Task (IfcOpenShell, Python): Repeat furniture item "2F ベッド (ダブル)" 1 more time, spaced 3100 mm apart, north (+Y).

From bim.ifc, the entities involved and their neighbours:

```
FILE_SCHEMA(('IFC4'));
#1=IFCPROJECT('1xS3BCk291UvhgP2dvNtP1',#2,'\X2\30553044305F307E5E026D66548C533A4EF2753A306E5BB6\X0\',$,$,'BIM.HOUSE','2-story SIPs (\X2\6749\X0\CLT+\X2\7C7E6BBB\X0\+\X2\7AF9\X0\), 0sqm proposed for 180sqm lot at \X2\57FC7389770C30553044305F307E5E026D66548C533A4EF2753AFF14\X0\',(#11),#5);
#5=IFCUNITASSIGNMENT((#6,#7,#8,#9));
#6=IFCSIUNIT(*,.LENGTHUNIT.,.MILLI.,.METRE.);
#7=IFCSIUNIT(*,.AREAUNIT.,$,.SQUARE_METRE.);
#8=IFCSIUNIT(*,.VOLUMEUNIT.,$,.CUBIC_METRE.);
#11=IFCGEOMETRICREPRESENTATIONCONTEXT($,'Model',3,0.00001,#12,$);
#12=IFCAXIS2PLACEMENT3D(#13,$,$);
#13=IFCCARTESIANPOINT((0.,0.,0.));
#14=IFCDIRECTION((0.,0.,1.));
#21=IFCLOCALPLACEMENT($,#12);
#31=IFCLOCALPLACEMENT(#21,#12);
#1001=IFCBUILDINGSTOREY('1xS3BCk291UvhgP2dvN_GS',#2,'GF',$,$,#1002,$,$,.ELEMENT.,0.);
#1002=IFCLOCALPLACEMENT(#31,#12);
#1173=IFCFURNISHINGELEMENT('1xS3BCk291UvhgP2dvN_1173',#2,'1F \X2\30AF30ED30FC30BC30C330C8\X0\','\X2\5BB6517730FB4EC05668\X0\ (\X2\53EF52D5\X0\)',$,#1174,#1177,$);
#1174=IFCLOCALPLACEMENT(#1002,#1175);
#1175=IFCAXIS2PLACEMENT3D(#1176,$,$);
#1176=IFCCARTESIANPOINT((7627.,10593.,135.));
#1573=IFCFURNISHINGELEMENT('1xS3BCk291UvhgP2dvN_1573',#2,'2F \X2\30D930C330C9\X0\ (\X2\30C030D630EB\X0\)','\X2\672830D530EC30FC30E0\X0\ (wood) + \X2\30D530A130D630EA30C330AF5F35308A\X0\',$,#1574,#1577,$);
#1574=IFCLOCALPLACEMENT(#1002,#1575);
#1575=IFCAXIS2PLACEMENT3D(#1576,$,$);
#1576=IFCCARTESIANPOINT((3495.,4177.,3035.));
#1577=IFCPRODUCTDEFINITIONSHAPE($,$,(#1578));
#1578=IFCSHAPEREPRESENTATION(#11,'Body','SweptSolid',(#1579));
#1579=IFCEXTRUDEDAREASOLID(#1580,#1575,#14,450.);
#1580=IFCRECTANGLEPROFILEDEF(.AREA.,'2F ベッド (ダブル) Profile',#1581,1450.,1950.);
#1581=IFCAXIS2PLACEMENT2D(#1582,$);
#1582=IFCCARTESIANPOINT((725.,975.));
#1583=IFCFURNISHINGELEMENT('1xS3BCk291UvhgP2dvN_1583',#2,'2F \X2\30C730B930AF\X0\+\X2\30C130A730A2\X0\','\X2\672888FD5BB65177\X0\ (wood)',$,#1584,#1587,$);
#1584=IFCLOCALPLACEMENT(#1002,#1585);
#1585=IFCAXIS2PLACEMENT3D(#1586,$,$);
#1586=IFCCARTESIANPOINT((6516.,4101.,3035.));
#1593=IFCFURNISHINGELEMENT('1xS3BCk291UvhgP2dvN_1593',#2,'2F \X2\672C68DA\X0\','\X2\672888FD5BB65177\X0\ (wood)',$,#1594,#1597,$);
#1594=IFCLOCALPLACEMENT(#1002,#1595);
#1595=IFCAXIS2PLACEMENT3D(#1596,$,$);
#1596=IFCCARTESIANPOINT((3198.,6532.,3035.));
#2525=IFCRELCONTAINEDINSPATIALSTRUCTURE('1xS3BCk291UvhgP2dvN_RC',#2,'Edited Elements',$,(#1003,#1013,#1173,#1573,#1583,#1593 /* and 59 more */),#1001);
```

```python
import numpy as np
import ifcopenshell
import ifcopenshell.api.geometry
import ifcopenshell.api.root
import ifcopenshell.util.element
import ifcopenshell.util.placement
import ifcopenshell.util.unit

model = ifcopenshell.open("bim.ifc")
unit_scale = ifcopenshell.util.unit.calculate_unit_scale(model)


def reuse_history(source, copy):
    """copy_class also copies each property set's owner history, people and application; keep the originals."""
    for rel in copy.IsDefinedBy:
        if rel.is_a("IfcRelDefinesByProperties") and (history := rel.RelatingPropertyDefinition.OwnerHistory):
            rel.RelatingPropertyDefinition.OwnerHistory = source.OwnerHistory
            ifcopenshell.util.element.remove_deep2(model, history)


source = model.by_guid("1xS3BCk291UvhgP2dvN_1573")
base = ifcopenshell.util.placement.get_local_placement(source.ObjectPlacement)
step = np.array([0.0, 1.0, 0.0]) * 3.1 / unit_scale

for i in range(1, 2):
    copy = ifcopenshell.api.root.copy_class(model, product=source)
    copy.Representation = ifcopenshell.util.element.copy_deep(
        model, source.Representation, exclude=["IfcGeometricRepresentationContext", "IfcRepresentationMap"]
    )
    reuse_history(source, copy)
    matrix = base.copy()
    matrix[:3, 3] += i * step
    print("added at", matrix[:3, 3].round(3) + 0.0)
    ifcopenshell.api.geometry.edit_object_placement(model, product=copy, matrix=matrix, is_si=False)

model.write("bim-out.ifc")
```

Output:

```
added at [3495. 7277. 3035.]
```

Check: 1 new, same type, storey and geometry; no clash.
